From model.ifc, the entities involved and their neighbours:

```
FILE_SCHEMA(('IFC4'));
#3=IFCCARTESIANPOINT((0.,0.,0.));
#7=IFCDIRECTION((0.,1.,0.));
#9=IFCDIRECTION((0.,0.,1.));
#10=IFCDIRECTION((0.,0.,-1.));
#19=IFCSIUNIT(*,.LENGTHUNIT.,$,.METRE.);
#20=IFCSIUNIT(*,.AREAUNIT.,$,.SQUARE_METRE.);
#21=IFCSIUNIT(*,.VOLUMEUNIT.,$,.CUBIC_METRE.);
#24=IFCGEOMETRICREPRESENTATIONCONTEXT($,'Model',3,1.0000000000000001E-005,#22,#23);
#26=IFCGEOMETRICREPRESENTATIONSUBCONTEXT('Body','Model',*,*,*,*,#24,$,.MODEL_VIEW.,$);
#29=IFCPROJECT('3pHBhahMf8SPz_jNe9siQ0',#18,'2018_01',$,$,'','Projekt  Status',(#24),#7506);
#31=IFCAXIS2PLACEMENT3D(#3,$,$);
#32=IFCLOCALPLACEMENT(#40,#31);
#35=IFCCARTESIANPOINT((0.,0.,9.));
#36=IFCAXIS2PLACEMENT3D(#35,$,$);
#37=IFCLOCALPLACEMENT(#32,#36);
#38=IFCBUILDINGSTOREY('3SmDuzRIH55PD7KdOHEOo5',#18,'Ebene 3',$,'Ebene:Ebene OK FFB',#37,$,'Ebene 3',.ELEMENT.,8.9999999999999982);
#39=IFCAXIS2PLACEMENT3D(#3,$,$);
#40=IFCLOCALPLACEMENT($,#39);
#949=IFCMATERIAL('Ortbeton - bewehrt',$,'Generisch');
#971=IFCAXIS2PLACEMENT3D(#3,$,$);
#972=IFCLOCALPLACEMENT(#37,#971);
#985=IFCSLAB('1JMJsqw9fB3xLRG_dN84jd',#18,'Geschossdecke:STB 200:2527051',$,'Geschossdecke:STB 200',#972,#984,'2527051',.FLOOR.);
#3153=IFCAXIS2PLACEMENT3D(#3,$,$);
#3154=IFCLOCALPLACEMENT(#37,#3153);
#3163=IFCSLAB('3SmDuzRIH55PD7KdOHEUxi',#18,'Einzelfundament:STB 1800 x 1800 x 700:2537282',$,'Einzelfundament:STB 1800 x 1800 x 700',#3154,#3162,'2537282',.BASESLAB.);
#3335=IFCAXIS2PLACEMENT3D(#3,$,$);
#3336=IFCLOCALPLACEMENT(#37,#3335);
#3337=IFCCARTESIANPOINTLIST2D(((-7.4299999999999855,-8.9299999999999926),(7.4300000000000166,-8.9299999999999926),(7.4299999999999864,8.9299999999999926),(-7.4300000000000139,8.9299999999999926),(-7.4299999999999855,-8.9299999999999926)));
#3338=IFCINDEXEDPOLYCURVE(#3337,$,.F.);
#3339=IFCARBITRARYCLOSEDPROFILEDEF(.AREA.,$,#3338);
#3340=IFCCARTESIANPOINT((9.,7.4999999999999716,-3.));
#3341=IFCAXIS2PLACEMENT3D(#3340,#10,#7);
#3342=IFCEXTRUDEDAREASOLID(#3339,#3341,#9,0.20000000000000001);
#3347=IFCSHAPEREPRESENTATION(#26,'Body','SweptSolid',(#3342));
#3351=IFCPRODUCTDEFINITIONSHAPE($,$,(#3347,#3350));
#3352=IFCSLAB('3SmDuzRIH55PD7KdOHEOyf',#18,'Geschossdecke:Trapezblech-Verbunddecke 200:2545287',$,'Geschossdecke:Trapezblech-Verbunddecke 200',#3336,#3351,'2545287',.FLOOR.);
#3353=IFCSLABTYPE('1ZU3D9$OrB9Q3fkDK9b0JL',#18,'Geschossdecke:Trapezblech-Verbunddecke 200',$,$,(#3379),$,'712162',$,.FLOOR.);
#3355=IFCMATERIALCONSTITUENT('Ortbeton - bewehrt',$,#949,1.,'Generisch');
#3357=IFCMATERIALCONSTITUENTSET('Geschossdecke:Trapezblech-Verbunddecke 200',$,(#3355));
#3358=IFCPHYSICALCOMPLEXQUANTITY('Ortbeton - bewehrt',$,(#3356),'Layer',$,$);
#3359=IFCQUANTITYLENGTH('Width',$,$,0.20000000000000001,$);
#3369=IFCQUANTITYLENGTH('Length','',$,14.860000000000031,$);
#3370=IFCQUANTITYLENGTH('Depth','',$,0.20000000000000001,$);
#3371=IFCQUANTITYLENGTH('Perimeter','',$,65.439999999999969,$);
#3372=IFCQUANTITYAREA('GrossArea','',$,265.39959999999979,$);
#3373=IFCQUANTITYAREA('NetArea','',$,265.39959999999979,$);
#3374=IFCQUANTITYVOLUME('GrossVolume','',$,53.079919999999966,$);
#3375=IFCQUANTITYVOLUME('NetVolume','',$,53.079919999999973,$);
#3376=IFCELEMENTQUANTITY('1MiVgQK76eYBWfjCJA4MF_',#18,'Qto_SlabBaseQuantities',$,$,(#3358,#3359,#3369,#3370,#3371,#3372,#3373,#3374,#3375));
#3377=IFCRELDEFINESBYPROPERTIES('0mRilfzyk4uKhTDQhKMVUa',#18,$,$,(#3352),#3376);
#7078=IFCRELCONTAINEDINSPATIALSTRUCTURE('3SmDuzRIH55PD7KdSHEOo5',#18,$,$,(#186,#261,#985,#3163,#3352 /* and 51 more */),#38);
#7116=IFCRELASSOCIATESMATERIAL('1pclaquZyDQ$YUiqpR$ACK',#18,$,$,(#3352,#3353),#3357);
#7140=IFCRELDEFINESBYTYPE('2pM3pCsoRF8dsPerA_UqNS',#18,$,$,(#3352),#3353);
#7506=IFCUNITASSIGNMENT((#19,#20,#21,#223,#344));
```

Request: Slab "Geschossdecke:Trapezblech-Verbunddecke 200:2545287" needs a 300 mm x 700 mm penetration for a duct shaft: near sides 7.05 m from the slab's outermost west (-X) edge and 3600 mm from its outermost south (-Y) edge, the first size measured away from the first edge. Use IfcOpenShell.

```python
import numpy as np
import ifcopenshell
import ifcopenshell.api.feature
import ifcopenshell.api.geometry
import ifcopenshell.api.pset
import ifcopenshell.api.root
import ifcopenshell.geom
import ifcopenshell.util.element
import ifcopenshell.util.placement
import ifcopenshell.util.representation
import ifcopenshell.util.shape
import ifcopenshell.util.unit

model = ifcopenshell.open("model.ifc")
unit_scale = ifcopenshell.util.unit.calculate_unit_scale(model)
area_scale = ifcopenshell.util.unit.calculate_unit_scale(model, "AREAUNIT")
volume_scale = ifcopenshell.util.unit.calculate_unit_scale(model, "VOLUMEUNIT")
settings = ifcopenshell.geom.settings()


def volume(element):
    """Net volume in cubic metres, openings subtracted."""
    shape = ifcopenshell.geom.create_shape(settings, element)
    return ifcopenshell.util.shape.get_volume(shape.geometry)


slab = model.by_guid("3SmDuzRIH55PD7KdOHEOyf")
before = volume(slab)

# Extent in the slab's own axes, in metres. The edges named are its -X and -Y sides.
slab_shape = ifcopenshell.geom.create_shape(settings, slab)
vertices = ifcopenshell.util.shape.get_vertices(slab_shape.geometry)
x_min, y_min, bottom = vertices.min(axis=0)
top = vertices[:, 2].max()

opening = ifcopenshell.api.root.create_entity(model, ifc_class="IfcOpeningElement", name="Duct shaft opening", predefined_type="OPENING")
context = ifcopenshell.util.representation.get_context(model, "Model", "Body", "MODEL_VIEW")
width, depth = 0.3, 0.7
outline = [(0.0, 0.0), (width, 0.0), (width, depth), (0.0, depth), (0.0, 0.0)]
# Overshoot both faces by 50 mm so the cut is clean.
shape = ifcopenshell.api.geometry.add_slab_representation(
    model, context=context, depth=top - bottom + 0.1, polyline=outline
)
ifcopenshell.api.geometry.assign_representation(model, product=opening, representation=shape)

matrix = ifcopenshell.util.placement.get_local_placement(slab.ObjectPlacement)
matrix[:, 3] = matrix @ np.append(np.array([x_min + 7.05, y_min + 3.6, bottom - 0.05]) / unit_scale, 1.0)
ifcopenshell.api.geometry.edit_object_placement(model, product=opening, matrix=matrix, is_si=False)
ifcopenshell.api.feature.add_feature(model, feature=opening, element=slab)

after = volume(slab)

# Update the slab's stored quantities.
qto = model.by_id(ifcopenshell.util.element.get_pset(slab, "Qto_SlabBaseQuantities", should_inherit=False)["id"])
ifcopenshell.api.pset.edit_qto(model, qto=qto, properties={
    "NetArea": after / (top - bottom) / area_scale,
    "NetVolume": after / volume_scale,
})

print(f"slab volume {before:.3f} -> {after:.3f} m3")

model.write("model-out.ifc")
```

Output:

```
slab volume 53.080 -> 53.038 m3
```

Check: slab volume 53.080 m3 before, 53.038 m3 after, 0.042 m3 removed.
